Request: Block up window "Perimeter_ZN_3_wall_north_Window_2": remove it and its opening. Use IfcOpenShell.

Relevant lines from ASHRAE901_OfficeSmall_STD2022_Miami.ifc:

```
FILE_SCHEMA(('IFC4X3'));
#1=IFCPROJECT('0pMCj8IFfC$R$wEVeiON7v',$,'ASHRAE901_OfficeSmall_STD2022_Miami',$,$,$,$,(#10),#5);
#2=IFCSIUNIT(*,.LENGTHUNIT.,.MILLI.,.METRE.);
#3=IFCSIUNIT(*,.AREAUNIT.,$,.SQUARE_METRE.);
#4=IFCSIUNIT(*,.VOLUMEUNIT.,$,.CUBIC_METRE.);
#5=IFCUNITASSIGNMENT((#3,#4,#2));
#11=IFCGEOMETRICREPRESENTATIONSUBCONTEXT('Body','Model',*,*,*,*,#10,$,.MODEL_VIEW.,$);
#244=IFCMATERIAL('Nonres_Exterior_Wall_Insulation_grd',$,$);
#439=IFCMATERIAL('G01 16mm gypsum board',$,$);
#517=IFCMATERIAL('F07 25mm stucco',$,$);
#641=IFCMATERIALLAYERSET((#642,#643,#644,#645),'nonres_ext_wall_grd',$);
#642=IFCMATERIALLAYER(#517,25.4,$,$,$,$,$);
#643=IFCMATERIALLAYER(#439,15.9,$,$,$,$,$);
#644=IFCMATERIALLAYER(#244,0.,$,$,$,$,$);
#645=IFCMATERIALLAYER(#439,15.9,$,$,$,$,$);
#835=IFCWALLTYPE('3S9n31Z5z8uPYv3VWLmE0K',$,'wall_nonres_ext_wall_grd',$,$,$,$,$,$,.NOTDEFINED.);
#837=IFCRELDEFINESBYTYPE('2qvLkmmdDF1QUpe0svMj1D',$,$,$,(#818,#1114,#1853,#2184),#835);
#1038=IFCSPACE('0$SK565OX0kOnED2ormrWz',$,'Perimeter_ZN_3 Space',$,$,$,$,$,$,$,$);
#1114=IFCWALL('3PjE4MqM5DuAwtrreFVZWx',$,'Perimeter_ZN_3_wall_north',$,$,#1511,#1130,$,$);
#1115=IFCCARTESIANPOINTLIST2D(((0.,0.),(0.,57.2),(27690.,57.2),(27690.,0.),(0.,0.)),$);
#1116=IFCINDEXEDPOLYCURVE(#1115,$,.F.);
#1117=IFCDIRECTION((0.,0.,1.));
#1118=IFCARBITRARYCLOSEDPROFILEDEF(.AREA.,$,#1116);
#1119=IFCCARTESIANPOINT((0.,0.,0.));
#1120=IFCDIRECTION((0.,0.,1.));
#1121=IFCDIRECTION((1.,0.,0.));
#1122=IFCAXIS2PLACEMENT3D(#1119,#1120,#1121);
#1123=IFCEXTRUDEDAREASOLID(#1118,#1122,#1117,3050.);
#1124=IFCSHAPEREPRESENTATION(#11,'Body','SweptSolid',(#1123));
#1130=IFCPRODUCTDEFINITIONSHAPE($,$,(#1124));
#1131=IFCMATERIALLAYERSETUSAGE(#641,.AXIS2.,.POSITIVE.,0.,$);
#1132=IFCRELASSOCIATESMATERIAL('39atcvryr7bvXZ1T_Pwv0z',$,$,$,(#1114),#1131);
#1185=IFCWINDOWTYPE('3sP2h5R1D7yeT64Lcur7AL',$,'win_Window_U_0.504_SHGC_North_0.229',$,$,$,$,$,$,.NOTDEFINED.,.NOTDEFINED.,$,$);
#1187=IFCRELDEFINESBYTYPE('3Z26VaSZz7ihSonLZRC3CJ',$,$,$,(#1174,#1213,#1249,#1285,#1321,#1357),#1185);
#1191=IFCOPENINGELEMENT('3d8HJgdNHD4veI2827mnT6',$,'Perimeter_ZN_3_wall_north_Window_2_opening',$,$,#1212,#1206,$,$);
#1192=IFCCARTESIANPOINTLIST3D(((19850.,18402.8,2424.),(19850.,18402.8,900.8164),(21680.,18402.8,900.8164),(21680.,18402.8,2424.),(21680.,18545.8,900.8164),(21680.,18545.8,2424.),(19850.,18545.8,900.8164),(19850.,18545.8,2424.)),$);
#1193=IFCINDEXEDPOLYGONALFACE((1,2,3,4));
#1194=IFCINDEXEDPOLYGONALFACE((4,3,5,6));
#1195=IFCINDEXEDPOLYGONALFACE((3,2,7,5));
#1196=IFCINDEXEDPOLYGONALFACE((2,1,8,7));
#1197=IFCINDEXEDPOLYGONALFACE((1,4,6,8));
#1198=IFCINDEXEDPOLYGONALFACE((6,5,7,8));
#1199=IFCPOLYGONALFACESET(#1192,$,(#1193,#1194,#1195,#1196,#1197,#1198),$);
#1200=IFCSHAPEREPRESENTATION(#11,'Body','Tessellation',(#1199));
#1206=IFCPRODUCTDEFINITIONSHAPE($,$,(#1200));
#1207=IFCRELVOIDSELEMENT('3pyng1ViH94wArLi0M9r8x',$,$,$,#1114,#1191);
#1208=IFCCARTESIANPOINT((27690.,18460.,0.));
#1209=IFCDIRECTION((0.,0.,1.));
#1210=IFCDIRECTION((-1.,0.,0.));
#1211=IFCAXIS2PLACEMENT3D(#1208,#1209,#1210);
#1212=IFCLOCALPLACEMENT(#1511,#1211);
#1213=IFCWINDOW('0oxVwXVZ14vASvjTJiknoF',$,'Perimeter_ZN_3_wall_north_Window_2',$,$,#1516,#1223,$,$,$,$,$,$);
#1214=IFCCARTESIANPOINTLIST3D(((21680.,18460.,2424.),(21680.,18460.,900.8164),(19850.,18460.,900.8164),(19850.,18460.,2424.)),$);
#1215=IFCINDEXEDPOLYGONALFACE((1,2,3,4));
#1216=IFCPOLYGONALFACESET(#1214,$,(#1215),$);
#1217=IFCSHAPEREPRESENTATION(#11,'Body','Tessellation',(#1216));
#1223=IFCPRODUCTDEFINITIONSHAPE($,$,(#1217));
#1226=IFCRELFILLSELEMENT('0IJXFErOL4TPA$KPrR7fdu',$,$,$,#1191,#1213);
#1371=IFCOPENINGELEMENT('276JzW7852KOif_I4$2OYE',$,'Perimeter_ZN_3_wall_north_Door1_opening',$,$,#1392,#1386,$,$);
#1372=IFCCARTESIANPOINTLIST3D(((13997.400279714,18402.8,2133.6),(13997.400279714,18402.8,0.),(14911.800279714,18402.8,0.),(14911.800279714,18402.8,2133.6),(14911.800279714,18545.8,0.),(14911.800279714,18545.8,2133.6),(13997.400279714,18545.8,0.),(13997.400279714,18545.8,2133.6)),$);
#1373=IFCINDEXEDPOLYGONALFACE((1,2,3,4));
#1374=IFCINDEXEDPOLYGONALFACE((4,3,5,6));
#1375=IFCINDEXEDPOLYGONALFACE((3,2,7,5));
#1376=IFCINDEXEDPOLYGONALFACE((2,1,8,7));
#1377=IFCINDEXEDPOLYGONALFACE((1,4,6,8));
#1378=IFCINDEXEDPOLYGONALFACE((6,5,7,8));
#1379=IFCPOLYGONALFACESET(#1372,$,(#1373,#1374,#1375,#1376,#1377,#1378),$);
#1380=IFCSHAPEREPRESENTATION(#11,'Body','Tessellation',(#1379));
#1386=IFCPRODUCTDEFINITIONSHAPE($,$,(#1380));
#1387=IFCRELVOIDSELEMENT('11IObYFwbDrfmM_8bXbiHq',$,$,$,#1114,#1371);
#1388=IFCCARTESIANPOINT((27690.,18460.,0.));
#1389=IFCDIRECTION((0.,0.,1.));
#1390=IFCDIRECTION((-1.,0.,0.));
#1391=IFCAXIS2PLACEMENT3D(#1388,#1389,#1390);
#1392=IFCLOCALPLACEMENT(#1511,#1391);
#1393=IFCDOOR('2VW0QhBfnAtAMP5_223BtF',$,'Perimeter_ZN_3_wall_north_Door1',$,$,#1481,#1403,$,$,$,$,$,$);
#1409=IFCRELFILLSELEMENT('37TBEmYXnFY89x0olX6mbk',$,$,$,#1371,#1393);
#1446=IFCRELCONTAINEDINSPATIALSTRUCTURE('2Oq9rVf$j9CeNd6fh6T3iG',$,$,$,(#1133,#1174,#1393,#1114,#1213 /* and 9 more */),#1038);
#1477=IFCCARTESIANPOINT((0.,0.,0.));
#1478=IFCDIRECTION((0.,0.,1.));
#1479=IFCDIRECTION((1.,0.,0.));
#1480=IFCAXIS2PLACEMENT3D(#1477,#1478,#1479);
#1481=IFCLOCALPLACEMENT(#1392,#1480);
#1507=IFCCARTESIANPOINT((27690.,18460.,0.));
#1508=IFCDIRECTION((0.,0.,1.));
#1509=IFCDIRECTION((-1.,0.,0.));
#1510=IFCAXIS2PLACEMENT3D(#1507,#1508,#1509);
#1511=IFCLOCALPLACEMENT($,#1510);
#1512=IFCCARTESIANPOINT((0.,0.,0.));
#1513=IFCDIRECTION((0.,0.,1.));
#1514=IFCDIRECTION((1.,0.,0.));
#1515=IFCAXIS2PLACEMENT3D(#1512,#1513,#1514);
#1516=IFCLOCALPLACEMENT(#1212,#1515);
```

```python
import ifcopenshell
import ifcopenshell.api.feature
import ifcopenshell.api.root
import ifcopenshell.geom
import ifcopenshell.util.shape

model = ifcopenshell.open("ASHRAE901_OfficeSmall_STD2022_Miami.ifc")
settings = ifcopenshell.geom.settings()


def volume(element):
    """Net volume in cubic metres, openings subtracted."""
    shape = ifcopenshell.geom.create_shape(settings, element)
    return ifcopenshell.util.shape.get_volume(shape.geometry)


window = model.by_guid("0oxVwXVZ14vASvjTJiknoF")
opening = window.FillsVoids[0].RelatingOpeningElement
wall = opening.VoidsElements[0].RelatingBuildingElement
before = volume(wall)

ifcopenshell.api.root.remove_product(model, product=window)
ifcopenshell.api.feature.remove_feature(model, feature=opening)

after = volume(wall)

print(f"wall volume {before:.3f} -> {after:.3f} m3")

model.write("ASHRAE901_OfficeSmall_STD2022_Miami_updated.ifc")
```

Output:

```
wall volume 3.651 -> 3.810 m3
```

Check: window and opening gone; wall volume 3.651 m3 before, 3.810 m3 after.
